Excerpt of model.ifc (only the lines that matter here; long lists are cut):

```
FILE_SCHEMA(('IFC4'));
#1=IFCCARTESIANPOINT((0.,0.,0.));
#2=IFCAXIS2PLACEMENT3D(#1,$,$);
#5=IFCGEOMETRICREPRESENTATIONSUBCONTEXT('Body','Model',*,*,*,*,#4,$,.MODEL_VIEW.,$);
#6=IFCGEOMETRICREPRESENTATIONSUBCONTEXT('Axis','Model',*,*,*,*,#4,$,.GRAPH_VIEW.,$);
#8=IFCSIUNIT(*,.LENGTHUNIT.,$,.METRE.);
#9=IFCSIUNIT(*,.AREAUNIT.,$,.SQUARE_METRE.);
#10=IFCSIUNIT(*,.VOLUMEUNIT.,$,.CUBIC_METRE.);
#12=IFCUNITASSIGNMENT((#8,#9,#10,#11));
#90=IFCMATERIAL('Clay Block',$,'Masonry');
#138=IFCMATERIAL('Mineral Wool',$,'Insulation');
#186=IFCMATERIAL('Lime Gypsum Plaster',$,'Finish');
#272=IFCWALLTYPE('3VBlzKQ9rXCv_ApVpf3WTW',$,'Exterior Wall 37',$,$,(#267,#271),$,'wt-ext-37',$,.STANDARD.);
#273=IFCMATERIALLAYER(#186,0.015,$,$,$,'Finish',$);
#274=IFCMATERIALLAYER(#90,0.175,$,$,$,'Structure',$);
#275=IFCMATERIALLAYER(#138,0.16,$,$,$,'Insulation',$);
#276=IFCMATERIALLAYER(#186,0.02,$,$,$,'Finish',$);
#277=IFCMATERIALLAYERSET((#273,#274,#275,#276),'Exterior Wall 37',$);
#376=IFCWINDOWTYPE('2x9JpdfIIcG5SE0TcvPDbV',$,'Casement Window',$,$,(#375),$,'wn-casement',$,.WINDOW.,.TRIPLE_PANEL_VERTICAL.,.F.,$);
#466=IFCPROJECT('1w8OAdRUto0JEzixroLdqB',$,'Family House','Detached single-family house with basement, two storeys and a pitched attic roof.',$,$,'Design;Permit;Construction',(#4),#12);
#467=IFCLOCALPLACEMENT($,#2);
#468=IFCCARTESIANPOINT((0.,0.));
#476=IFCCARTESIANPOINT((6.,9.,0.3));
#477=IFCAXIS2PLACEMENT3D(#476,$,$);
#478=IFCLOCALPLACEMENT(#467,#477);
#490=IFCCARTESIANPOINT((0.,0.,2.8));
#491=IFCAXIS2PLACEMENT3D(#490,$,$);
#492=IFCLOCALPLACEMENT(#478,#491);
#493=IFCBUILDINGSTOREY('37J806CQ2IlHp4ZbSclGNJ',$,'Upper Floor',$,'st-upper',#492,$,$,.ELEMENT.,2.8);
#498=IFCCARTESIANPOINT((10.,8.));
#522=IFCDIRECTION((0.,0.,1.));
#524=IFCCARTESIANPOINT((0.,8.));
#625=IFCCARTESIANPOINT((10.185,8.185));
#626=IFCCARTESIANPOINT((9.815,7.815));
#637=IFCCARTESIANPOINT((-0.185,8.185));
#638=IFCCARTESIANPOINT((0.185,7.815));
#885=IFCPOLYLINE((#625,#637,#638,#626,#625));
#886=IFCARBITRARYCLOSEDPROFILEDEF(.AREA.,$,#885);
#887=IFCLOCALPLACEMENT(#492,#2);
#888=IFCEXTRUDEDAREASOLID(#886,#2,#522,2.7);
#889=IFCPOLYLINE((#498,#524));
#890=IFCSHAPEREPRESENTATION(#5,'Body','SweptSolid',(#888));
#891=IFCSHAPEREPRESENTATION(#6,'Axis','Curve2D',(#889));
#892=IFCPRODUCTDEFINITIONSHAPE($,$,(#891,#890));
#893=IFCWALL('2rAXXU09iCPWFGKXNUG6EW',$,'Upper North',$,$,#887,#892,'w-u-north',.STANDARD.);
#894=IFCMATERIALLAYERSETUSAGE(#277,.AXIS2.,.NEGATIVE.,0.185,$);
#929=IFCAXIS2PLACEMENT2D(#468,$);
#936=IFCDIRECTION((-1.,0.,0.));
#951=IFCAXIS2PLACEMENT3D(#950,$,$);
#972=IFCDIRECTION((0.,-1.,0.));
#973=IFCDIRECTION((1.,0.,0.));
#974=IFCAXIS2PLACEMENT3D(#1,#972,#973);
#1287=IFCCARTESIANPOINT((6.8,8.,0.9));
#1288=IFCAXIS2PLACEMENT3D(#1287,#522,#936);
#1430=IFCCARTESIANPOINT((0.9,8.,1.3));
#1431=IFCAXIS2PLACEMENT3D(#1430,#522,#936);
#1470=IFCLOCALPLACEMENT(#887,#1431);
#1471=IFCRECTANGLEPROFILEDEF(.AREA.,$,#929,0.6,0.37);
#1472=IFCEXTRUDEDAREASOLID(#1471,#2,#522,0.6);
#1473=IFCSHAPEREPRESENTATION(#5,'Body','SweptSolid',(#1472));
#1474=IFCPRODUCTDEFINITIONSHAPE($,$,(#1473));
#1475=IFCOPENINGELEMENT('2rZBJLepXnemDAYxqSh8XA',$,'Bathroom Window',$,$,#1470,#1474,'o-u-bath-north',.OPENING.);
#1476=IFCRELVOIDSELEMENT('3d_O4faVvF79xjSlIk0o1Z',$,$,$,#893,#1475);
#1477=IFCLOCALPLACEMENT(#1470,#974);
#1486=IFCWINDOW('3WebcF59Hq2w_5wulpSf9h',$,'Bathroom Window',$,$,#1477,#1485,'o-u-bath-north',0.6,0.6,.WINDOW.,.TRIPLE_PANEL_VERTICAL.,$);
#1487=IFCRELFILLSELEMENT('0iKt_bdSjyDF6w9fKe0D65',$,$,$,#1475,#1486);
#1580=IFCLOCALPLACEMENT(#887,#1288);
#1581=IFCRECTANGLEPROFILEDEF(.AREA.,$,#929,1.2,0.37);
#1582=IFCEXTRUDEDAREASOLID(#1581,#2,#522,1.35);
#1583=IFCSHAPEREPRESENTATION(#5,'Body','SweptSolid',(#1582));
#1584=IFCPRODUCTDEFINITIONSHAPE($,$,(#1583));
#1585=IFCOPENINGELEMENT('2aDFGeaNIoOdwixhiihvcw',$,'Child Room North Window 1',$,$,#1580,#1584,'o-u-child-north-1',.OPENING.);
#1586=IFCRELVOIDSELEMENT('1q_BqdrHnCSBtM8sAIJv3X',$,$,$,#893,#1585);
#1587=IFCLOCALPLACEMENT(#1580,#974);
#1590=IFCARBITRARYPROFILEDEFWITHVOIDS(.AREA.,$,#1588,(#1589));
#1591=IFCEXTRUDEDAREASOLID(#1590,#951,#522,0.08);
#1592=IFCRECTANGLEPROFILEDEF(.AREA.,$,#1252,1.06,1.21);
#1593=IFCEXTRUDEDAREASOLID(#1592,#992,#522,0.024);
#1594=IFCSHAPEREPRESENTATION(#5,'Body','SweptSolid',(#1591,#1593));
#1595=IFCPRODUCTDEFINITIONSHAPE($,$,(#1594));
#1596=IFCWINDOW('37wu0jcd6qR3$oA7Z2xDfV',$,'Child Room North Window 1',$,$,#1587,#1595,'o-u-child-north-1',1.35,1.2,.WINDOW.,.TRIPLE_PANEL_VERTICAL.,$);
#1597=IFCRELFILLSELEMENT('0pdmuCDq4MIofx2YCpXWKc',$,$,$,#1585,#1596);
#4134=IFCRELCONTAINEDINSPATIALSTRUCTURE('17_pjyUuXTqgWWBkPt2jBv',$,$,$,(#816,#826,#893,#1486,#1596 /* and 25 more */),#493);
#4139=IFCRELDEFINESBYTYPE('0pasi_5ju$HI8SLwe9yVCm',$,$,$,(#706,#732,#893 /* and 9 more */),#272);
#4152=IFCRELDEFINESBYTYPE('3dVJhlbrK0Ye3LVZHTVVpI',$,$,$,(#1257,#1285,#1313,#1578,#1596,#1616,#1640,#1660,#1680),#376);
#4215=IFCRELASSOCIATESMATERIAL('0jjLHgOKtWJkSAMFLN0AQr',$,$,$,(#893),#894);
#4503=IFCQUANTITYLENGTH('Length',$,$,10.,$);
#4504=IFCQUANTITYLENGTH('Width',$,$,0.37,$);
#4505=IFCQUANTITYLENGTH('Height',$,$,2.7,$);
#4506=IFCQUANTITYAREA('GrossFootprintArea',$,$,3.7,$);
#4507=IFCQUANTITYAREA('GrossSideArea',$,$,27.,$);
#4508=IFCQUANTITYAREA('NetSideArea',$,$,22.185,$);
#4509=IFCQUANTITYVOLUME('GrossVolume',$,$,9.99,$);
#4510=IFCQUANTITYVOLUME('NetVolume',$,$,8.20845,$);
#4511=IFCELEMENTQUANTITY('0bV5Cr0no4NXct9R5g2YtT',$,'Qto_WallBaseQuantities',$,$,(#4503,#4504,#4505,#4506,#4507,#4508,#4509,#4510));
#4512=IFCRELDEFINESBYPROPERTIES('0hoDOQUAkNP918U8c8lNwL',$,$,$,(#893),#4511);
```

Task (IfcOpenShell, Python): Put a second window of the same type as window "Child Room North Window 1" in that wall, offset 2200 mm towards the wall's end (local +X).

```python
import ifcopenshell
import ifcopenshell.api.feature
import ifcopenshell.api.geometry
import ifcopenshell.api.pset
import ifcopenshell.api.root
import ifcopenshell.geom
import ifcopenshell.util.element
import ifcopenshell.util.placement
import ifcopenshell.util.shape
import ifcopenshell.util.unit

model = ifcopenshell.open("model.ifc")
unit_scale = ifcopenshell.util.unit.calculate_unit_scale(model)
area_scale = ifcopenshell.util.unit.calculate_unit_scale(model, "AREAUNIT")
volume_scale = ifcopenshell.util.unit.calculate_unit_scale(model, "VOLUMEUNIT")
settings = ifcopenshell.geom.settings()


def volume(element):
    """Net volume in cubic metres, openings subtracted."""
    shape = ifcopenshell.geom.create_shape(settings, element)
    return ifcopenshell.util.shape.get_volume(shape.geometry)


window = model.by_id(1596)
opening = window.FillsVoids[0].RelatingOpeningElement
wall = opening.VoidsElements[0].RelatingBuildingElement
before = volume(wall)
shift = ifcopenshell.util.placement.get_local_placement(wall.ObjectPlacement)[:3, 0] * 2.2 / unit_scale

# copy_class copies the void relationship, type, container and properties, but no geometry.
new_opening = ifcopenshell.api.root.copy_class(model, product=opening)
new_opening.Representation = ifcopenshell.util.element.copy_deep(
    model, opening.Representation, exclude=["IfcGeometricRepresentationContext", "IfcRepresentationMap"]
)
new_opening.Tag = None
new_window = ifcopenshell.api.root.copy_class(model, product=window)
new_window.Representation = ifcopenshell.util.element.copy_deep(
    model, window.Representation, exclude=["IfcGeometricRepresentationContext", "IfcRepresentationMap"]
)
new_window.Tag = None
ifcopenshell.api.feature.add_filling(model, opening=new_opening, element=new_window)

for old, new in ((opening, new_opening), (window, new_window)):
    matrix = ifcopenshell.util.placement.get_local_placement(old.ObjectPlacement)
    matrix[:3, 3] += shift
    ifcopenshell.api.geometry.edit_object_placement(model, product=new, matrix=matrix, is_si=False)

after = volume(wall)
thickness = 0.37  # wall thickness in metres

# Update the wall's stored quantities.
qto = model.by_id(ifcopenshell.util.element.get_pset(wall, "Qto_WallBaseQuantities", should_inherit=False)["id"])
ifcopenshell.api.pset.edit_qto(model, qto=qto, properties={
    "NetSideArea": after / thickness / area_scale,
    "NetVolume": after / volume_scale,
})

print(f"wall volume {before:.3f} -> {after:.3f} m3")

model.write("model-out.ifc")
```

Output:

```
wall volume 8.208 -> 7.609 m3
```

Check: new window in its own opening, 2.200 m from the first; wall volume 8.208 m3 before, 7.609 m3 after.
